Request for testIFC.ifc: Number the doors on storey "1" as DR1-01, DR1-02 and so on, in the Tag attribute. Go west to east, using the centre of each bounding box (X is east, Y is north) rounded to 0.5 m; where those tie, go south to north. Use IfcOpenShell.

First a look at what the model holds.

```python
import ifcopenshell
import ifcopenshell.util.element
import ifcopenshell.util.placement

model = ifcopenshell.open("testIFC.ifc")
print(model.schema)
storey = next(s for s in model.by_type("IfcBuildingStorey") if s.Name == "1")
doors = [e for e in ifcopenshell.util.element.get_decomposition(storey) if e.is_a("IfcDoor")]
for e in sorted(doors, key=lambda e: e.id()):
    origin = ifcopenshell.util.placement.get_local_placement(e.ObjectPlacement)[:3, 3]
    print(e.id(), e.Tag, e.Name, origin.round(2) + 0.0, sep=" | ")
```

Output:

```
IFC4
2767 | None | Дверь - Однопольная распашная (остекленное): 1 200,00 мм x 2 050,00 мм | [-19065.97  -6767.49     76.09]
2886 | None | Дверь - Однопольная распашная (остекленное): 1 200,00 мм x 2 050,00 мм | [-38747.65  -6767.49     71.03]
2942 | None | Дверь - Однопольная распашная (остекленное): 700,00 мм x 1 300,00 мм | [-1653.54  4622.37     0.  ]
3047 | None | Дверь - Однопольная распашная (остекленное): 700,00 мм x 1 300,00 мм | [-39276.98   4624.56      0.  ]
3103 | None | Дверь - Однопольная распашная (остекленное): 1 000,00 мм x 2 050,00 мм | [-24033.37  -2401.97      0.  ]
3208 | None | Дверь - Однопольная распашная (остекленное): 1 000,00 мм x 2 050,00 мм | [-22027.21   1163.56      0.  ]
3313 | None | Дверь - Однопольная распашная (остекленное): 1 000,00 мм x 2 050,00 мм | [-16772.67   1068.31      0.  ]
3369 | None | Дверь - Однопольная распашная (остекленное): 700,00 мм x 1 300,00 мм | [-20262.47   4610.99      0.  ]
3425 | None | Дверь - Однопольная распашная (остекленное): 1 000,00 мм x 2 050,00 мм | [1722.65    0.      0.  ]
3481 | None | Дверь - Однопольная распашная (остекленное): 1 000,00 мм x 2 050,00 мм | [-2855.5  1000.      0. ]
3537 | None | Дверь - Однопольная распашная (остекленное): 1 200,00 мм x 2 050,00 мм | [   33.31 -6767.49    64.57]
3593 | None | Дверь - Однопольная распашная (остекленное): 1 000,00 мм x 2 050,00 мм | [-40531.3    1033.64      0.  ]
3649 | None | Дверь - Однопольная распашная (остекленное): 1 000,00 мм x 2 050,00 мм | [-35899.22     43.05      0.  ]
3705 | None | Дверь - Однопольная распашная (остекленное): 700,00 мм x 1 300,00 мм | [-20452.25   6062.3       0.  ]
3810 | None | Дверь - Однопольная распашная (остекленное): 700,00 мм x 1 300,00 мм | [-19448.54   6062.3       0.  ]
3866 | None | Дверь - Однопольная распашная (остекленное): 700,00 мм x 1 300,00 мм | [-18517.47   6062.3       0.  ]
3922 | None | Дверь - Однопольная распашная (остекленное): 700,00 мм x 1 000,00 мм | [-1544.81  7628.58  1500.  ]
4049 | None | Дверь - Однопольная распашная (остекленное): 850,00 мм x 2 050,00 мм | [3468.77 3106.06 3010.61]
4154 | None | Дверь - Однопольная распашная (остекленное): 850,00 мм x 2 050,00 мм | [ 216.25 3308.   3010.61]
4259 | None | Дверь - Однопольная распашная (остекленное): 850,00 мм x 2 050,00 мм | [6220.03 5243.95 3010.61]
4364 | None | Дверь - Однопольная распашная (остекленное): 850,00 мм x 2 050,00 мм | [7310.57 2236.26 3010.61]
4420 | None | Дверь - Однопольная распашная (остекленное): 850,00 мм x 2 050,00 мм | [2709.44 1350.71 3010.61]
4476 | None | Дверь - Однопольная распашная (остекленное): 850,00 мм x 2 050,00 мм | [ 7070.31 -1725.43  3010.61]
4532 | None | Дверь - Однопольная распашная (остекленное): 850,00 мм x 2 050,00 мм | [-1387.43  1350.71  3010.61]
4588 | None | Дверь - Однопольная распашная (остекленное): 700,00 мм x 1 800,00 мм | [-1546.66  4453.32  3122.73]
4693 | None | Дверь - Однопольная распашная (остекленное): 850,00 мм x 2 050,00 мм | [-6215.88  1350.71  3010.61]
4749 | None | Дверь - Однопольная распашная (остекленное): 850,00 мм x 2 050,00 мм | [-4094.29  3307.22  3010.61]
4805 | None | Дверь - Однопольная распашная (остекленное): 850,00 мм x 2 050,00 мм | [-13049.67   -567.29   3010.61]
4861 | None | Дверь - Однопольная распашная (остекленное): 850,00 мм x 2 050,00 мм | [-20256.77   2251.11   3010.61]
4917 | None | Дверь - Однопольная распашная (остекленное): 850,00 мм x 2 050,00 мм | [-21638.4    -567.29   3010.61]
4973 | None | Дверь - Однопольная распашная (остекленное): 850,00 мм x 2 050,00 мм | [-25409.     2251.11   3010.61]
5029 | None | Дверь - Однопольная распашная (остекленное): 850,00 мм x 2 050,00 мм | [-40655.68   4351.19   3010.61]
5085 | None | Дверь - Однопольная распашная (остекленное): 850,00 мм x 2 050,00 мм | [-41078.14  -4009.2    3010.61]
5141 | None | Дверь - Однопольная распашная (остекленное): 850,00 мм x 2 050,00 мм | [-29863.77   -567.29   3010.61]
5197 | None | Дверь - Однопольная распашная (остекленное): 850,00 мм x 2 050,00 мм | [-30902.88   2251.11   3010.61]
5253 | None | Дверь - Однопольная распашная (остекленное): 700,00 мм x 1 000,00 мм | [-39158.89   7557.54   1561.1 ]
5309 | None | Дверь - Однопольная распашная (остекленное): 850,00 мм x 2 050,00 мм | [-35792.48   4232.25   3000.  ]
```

```python
import ifcopenshell
import ifcopenshell.geom
import ifcopenshell.util.element
import ifcopenshell.util.shape

model = ifcopenshell.open("testIFC.ifc")
settings = ifcopenshell.geom.settings()
settings.set("use-world-coords", True)


def centre(element):
    shape = ifcopenshell.geom.create_shape(settings, element)
    return ifcopenshell.util.shape.get_bbox_centroid(shape.geometry)


storey = next(s for s in model.by_type("IfcBuildingStorey") if s.Name == "1")
doors = [e for e in ifcopenshell.util.element.get_decomposition(storey) if e.is_a("IfcDoor")]

# Insertion points can sit at a corner or the storey origin, so sort by the geometry (in metres).
centres = {e: centre(e) for e in doors}
doors.sort(key=lambda e: (round(centres[e][0] / 0.5), centres[e][1]))

for i, e in enumerate(doors, start=1):
    number = f"DR1-{i:02d}"
    e.Tag = number
    print(e.id(), number)

model.write("testIFC_rev.ifc")
```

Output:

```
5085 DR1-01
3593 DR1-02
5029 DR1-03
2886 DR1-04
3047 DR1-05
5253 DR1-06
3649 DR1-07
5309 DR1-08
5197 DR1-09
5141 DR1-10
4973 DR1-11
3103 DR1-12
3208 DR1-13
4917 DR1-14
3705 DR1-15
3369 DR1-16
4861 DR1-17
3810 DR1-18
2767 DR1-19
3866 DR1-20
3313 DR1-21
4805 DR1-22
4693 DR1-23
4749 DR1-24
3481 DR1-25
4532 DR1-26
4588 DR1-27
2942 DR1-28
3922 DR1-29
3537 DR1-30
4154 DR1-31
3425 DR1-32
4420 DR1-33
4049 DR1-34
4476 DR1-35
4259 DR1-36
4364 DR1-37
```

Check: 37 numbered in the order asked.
